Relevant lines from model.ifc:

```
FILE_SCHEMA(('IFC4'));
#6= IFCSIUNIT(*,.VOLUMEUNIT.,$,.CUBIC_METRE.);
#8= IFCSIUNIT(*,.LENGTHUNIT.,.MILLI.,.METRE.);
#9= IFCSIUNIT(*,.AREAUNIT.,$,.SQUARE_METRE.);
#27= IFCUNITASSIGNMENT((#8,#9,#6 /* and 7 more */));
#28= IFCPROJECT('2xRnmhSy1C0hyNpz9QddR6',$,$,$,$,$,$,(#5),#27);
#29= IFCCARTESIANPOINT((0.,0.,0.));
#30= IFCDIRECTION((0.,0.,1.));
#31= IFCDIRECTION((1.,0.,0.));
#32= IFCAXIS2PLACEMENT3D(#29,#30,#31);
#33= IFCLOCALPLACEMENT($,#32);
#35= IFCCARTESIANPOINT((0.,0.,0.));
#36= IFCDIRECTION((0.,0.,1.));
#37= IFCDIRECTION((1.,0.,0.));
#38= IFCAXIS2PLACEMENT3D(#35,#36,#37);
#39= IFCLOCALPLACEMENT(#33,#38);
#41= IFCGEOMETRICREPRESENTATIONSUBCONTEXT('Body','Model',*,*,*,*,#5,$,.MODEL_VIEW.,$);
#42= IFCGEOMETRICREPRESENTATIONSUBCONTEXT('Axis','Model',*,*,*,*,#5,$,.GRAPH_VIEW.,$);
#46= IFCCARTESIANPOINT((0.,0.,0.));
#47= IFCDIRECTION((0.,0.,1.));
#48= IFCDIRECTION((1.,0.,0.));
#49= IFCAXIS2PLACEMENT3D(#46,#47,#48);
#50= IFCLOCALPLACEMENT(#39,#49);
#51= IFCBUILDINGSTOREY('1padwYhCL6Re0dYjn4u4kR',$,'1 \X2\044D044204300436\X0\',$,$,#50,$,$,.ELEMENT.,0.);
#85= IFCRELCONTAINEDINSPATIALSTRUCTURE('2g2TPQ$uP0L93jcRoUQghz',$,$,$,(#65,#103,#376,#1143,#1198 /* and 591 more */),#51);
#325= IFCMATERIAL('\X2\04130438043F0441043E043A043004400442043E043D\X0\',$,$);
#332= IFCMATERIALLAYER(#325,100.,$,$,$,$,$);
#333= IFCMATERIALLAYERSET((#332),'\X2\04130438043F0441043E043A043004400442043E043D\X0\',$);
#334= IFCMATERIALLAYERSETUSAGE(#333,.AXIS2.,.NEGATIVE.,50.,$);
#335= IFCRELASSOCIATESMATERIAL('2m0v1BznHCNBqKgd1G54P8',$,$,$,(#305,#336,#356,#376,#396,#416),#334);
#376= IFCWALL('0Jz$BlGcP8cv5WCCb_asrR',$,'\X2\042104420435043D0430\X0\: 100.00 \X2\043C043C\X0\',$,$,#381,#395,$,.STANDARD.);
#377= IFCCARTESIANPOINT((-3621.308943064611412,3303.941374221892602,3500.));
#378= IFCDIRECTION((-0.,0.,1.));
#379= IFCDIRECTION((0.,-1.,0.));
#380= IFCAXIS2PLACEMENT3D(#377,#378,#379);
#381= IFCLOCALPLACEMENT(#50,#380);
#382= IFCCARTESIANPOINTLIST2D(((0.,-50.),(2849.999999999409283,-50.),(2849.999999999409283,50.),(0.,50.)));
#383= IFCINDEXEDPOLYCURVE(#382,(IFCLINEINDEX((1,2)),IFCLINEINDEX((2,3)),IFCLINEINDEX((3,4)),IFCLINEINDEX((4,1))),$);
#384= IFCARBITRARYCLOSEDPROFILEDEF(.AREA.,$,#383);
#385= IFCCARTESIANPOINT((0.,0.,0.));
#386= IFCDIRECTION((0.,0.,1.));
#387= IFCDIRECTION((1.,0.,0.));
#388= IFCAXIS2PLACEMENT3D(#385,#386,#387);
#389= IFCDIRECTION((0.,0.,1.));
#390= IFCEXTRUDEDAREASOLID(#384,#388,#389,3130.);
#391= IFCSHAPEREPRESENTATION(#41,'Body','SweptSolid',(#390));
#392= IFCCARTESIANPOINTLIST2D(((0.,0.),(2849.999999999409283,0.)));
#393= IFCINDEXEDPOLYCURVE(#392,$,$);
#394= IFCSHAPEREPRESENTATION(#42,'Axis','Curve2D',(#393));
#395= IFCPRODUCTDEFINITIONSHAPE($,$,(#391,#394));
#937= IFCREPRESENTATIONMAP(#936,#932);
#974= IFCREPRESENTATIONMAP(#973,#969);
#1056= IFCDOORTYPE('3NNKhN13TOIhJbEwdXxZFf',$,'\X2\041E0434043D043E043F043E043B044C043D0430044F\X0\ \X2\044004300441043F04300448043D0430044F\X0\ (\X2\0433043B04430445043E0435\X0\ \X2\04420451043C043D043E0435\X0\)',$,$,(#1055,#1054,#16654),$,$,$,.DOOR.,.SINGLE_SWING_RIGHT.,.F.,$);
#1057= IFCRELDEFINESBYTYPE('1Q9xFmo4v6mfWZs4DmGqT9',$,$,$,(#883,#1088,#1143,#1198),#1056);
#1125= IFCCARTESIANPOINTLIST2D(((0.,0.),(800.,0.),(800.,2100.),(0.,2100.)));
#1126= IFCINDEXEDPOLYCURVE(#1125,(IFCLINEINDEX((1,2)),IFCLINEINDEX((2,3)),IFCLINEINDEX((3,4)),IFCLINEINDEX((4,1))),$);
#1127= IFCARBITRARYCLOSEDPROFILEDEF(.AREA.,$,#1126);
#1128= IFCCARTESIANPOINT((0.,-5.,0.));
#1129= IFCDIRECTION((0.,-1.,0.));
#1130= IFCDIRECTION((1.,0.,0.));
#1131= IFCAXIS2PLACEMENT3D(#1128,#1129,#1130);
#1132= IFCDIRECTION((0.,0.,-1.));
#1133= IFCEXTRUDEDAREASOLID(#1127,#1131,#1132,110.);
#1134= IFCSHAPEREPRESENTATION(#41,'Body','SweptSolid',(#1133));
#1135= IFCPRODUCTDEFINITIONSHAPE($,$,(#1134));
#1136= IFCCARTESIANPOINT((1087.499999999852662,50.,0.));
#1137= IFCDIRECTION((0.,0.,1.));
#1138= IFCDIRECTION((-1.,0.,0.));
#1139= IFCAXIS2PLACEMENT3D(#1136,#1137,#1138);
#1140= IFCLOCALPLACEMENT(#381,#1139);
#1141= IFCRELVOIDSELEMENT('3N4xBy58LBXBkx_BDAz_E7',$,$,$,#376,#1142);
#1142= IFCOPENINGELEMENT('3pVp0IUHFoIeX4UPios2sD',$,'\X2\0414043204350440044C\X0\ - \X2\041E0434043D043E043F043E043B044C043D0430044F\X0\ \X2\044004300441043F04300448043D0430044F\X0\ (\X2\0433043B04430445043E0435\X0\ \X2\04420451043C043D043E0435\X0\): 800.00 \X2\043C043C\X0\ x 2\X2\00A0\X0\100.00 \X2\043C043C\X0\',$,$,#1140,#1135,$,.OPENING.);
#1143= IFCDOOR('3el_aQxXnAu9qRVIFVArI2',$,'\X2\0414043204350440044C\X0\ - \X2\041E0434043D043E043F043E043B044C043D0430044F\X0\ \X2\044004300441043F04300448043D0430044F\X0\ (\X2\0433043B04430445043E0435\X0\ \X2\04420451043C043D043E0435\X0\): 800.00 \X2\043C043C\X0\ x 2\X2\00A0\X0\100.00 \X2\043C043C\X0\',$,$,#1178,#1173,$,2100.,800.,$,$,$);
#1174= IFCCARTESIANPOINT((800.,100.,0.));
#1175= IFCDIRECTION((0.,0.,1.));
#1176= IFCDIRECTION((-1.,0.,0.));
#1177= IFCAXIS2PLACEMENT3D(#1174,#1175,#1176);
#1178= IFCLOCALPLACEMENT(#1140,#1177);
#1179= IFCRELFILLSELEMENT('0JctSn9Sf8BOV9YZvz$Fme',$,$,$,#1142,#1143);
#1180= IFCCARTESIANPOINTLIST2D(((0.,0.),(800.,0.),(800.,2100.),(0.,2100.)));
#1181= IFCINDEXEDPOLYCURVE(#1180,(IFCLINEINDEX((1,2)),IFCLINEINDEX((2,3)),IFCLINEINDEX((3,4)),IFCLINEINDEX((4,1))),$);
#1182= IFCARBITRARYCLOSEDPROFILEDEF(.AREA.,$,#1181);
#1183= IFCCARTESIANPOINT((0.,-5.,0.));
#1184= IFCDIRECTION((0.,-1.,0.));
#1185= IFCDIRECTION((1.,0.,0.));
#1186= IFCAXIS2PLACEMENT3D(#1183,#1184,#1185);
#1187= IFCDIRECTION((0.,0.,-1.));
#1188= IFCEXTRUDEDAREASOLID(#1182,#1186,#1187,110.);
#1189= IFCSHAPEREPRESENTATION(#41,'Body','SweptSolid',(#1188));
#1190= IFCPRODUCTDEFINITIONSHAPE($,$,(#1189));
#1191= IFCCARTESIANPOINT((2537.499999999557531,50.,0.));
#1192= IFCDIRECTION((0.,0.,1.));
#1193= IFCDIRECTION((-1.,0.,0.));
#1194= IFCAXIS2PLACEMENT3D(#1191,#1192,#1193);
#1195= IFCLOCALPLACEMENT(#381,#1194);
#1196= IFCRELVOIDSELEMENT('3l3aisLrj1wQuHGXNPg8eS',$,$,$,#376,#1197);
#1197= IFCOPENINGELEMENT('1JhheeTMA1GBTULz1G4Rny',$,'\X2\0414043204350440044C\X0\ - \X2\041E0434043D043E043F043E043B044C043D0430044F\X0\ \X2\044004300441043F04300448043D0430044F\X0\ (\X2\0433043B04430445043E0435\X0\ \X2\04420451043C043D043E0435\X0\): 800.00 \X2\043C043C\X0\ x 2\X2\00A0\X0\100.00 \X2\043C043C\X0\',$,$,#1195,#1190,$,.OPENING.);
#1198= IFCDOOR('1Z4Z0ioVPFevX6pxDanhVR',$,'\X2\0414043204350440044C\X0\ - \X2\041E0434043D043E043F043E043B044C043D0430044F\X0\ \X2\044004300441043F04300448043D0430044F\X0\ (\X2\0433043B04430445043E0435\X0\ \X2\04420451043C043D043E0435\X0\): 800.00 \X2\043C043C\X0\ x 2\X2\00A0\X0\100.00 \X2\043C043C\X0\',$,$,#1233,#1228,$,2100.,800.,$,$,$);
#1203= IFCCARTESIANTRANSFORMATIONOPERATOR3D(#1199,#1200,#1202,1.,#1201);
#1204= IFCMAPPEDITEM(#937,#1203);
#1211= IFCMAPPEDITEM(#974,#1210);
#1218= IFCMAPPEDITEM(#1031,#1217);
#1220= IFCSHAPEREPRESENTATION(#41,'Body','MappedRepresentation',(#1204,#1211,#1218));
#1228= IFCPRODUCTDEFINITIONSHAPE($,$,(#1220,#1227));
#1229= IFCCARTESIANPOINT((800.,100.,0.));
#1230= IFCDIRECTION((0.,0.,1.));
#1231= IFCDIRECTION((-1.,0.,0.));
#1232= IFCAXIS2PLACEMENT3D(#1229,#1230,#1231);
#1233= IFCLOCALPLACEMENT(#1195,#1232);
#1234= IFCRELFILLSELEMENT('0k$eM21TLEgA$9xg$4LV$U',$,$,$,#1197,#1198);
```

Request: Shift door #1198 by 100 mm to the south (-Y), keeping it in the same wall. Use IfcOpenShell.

```python
import ifcopenshell
import ifcopenshell.api.geometry
import ifcopenshell.util.placement
import ifcopenshell.util.unit

model = ifcopenshell.open("model.ifc")
unit_scale = ifcopenshell.util.unit.calculate_unit_scale(model)

door = model.by_id(1198)
opening = door.FillsVoids[0].RelatingOpeningElement
wall = opening.VoidsElements[0].RelatingBuildingElement

wall_matrix = ifcopenshell.util.placement.get_local_placement(wall.ObjectPlacement)
shift = wall_matrix[:3, 0] * 0.1 / unit_scale
before = ifcopenshell.util.placement.get_local_placement(door.ObjectPlacement)[:3, 3].copy()

# The door is placed relative to its opening, so it follows when the opening moves.
matrix = ifcopenshell.util.placement.get_local_placement(opening.ObjectPlacement)
matrix[:3, 3] += shift
ifcopenshell.api.geometry.edit_object_placement(
    model, product=opening, matrix=matrix, is_si=False, should_transform_children=True
)

after = ifcopenshell.util.placement.get_local_placement(door.ObjectPlacement)[:3, 3]
print("door moved by", (after - before).round(3) + 0.0)

model.write("model_edited.ifc")
```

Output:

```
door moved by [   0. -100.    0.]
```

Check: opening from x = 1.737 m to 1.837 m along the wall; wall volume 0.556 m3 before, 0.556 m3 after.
